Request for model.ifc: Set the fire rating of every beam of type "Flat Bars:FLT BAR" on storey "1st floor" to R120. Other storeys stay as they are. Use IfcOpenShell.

First a look at what the model holds.

```python
import ifcopenshell
import ifcopenshell.util.element

model = ifcopenshell.open("model.ifc")
print(model.schema)
storey = next(s for s in model.by_type("IfcBuildingStorey") if s.Name == "1st floor")
beams = [e for e in ifcopenshell.util.element.get_decomposition(storey) if e.is_a("IfcBeam")]
seen = {}
for e in beams:
    element_type = ifcopenshell.util.element.get_type(e)
    key = (element_type.Name if element_type != e and element_type else None, ifcopenshell.util.element.get_pset(e, "Pset_BeamCommon", "FireRating"))
    seen[key] = seen.get(key, 0) + 1
for (name, value), count in sorted(seen.items(), key=str):
    print(count, "x", name, "|", value)
```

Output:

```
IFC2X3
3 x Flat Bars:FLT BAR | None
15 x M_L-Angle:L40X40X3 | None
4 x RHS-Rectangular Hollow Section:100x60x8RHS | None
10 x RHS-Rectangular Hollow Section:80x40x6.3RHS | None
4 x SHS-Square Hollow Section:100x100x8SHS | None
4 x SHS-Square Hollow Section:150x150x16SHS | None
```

```python
import ifcopenshell
import ifcopenshell.api.pset
import ifcopenshell.util.element

model = ifcopenshell.open("model.ifc")

storey = next(s for s in model.by_type("IfcBuildingStorey") if s.Name == "1st floor")
beams = [e for e in ifcopenshell.util.element.get_decomposition(storey) if e.is_a("IfcBeam")]

count = 0
for e in beams:
    element_type = ifcopenshell.util.element.get_type(e)
    if element_type in (None, e) or element_type.Name != "Flat Bars:FLT BAR":
        continue
    # add_pset returns the element's existing set when there is one.
    pset = ifcopenshell.api.pset.add_pset(model, product=e, name="Pset_BeamCommon")
    ifcopenshell.api.pset.edit_pset(model, pset=pset, properties={"FireRating": "R120"})
    count += 1

print(count, "beams updated")

model.write("model_v2.ifc")
```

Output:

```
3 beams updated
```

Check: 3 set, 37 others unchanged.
